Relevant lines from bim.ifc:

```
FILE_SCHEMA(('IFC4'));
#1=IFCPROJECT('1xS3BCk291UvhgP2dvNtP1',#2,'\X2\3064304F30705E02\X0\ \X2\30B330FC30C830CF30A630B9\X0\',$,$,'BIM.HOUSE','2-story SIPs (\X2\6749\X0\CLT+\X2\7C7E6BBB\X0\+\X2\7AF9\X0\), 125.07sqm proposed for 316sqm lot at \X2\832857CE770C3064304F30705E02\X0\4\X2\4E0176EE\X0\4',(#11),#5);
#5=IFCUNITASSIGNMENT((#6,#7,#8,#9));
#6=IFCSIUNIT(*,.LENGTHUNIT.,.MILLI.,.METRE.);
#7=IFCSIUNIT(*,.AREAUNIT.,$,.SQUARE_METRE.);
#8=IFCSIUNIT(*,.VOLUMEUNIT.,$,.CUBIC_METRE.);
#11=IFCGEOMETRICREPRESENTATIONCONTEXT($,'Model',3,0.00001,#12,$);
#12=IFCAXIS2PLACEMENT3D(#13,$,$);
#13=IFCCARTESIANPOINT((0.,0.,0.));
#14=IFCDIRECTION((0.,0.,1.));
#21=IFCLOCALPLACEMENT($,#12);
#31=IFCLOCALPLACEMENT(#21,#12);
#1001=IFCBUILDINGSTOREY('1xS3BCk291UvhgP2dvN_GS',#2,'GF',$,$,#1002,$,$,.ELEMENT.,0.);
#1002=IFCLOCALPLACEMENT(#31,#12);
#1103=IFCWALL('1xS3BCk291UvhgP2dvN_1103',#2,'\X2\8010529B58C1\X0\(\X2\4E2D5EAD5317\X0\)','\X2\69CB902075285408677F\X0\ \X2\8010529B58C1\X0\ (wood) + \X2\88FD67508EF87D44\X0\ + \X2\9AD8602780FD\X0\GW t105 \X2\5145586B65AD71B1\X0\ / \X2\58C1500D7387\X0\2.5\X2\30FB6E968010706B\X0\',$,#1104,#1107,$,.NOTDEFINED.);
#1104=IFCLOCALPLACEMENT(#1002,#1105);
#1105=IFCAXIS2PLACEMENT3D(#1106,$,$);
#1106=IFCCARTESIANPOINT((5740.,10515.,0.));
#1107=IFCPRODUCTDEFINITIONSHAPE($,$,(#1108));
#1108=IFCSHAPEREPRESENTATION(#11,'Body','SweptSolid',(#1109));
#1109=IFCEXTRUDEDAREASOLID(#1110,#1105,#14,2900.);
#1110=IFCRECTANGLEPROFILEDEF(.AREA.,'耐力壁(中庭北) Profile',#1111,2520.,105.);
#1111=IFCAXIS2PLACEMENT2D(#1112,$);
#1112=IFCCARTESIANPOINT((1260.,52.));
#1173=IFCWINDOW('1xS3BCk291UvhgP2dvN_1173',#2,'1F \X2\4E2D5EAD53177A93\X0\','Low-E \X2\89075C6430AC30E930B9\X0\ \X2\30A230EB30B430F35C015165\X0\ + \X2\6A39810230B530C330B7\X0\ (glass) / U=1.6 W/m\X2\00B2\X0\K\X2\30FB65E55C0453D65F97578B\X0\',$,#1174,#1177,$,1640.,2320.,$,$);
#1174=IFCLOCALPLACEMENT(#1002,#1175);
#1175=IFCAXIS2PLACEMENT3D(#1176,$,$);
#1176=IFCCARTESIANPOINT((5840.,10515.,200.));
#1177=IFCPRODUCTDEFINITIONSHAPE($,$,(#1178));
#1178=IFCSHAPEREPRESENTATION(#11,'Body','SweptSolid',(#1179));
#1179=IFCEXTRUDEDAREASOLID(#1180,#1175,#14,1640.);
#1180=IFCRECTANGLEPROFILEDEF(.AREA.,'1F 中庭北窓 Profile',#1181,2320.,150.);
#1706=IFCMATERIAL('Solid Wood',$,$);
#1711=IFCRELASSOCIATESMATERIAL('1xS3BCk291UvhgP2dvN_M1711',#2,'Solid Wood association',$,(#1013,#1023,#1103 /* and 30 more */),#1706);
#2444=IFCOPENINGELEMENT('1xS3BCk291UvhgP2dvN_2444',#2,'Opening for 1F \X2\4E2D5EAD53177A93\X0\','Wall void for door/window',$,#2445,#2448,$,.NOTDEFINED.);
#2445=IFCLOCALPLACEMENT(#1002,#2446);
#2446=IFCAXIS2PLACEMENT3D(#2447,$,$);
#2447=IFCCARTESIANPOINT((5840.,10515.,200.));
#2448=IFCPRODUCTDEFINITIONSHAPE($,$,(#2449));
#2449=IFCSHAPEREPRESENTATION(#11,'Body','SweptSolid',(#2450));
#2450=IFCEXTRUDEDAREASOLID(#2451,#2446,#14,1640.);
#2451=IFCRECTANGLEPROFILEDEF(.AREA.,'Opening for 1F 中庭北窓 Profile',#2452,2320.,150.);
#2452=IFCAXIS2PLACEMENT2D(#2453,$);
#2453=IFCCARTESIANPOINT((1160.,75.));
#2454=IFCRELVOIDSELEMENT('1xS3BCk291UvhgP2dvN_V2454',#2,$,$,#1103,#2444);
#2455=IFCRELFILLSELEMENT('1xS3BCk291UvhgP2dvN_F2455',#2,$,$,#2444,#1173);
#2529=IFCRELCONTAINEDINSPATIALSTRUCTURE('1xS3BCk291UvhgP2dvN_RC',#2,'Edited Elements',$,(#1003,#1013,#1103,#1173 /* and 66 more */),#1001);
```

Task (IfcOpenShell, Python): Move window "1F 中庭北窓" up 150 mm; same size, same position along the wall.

```python
import numpy as np
import ifcopenshell
import ifcopenshell.api.geometry
import ifcopenshell.util.placement
import ifcopenshell.util.unit

model = ifcopenshell.open("bim.ifc")
unit_scale = ifcopenshell.util.unit.calculate_unit_scale(model)

window = model.by_id(1173)
opening = window.FillsVoids[0].RelatingOpeningElement
dz = 150.0

shift = np.array([0.0, 0.0, dz])
# The window is not placed relative to its opening, so move both.
for product in (opening, window):
    matrix = ifcopenshell.util.placement.get_local_placement(product.ObjectPlacement)
    matrix[:3, 3] += shift
    ifcopenshell.api.geometry.edit_object_placement(model, product=product, matrix=matrix, is_si=False)

print(f"moved by {dz * unit_scale:+.3f} m")

model.write("bim_rev.ifc")
```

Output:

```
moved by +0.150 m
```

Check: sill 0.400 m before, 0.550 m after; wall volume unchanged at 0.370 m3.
